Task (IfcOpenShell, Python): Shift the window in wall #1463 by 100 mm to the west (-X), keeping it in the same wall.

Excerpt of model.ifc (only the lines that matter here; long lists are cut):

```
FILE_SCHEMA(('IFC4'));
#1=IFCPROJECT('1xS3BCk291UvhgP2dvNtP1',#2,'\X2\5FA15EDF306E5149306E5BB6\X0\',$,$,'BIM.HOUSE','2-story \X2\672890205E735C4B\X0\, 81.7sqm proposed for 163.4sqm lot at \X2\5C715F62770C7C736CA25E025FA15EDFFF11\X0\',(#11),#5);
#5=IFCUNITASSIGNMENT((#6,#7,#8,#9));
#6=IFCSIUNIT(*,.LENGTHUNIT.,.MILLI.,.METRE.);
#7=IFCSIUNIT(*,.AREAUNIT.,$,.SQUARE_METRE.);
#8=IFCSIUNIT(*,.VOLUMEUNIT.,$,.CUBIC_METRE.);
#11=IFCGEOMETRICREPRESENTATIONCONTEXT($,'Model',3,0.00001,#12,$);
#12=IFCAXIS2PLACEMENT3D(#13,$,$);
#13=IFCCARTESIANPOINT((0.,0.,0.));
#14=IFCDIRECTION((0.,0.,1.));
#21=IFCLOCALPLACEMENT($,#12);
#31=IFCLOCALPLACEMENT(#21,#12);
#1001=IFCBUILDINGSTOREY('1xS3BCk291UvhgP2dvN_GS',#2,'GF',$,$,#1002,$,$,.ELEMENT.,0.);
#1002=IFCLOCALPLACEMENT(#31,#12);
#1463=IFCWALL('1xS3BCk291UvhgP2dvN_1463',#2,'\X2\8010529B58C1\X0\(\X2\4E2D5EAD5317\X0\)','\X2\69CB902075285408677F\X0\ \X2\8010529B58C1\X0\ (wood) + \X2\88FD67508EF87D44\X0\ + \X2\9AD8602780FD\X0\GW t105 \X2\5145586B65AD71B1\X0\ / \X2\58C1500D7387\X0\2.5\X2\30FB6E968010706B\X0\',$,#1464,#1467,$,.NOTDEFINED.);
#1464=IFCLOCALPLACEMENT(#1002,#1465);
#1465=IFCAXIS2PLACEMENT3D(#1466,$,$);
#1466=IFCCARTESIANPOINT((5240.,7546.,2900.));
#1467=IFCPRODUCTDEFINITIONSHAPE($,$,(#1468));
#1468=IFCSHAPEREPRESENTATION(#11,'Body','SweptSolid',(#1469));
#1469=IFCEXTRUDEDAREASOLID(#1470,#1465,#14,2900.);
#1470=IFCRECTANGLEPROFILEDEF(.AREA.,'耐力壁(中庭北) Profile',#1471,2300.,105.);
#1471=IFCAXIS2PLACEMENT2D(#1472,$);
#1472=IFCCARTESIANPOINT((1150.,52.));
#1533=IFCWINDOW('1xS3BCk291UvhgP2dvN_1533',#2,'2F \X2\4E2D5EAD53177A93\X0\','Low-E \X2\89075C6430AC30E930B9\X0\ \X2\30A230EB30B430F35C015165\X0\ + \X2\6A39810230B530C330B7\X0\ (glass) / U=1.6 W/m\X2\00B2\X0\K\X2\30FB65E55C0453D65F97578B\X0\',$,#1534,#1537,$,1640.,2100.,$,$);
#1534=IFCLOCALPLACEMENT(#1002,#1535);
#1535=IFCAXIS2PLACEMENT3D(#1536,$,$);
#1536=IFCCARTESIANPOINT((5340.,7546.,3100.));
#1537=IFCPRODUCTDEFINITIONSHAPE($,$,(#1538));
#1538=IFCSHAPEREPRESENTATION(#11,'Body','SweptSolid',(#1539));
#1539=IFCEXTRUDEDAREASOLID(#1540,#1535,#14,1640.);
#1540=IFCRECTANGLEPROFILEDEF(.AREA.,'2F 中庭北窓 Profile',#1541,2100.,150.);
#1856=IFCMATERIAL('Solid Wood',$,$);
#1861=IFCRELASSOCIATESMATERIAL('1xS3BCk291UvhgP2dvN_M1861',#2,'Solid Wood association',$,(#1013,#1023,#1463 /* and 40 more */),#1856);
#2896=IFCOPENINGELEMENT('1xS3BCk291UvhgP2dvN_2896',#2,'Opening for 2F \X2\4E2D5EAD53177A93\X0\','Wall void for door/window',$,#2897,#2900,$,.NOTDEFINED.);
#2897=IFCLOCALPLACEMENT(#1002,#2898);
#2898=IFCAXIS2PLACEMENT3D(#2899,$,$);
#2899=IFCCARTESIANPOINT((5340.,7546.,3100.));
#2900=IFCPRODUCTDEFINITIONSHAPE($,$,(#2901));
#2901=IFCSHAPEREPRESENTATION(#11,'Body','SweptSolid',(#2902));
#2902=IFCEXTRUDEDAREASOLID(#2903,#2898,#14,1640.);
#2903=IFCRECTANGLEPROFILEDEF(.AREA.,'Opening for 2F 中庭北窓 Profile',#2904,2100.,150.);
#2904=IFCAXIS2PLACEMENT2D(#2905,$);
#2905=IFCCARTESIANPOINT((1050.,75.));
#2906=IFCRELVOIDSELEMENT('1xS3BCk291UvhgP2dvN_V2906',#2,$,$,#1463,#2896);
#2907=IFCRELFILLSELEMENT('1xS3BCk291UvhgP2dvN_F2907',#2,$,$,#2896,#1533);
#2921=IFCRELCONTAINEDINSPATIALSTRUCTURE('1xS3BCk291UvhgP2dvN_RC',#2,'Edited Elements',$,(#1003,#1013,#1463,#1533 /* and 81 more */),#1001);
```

```python
import ifcopenshell
import ifcopenshell.api.geometry
import ifcopenshell.util.placement
import ifcopenshell.util.unit

model = ifcopenshell.open("model.ifc")
unit_scale = ifcopenshell.util.unit.calculate_unit_scale(model)

window = model.by_guid("1xS3BCk291UvhgP2dvN_1533")
opening = window.FillsVoids[0].RelatingOpeningElement
wall = opening.VoidsElements[0].RelatingBuildingElement

wall_matrix = ifcopenshell.util.placement.get_local_placement(wall.ObjectPlacement)
shift = wall_matrix[:3, 0] * -0.1 / unit_scale
before = ifcopenshell.util.placement.get_local_placement(window.ObjectPlacement)[:3, 3].copy()

# The window is not placed relative to its opening, so move both.
for product in (opening, window):
    matrix = ifcopenshell.util.placement.get_local_placement(product.ObjectPlacement)
    matrix[:3, 3] += shift
    ifcopenshell.api.geometry.edit_object_placement(model, product=product, matrix=matrix, is_si=False)

after = ifcopenshell.util.placement.get_local_placement(window.ObjectPlacement)[:3, 3]
print("window moved by", (after - before).round(3) + 0.0)

model.write("model_updated.ifc")
```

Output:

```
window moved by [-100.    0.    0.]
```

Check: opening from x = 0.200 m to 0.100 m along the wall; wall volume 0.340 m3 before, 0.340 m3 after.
